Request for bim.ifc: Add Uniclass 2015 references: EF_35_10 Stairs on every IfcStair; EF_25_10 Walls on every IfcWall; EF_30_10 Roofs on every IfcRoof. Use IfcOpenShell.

First a look at what the model holds.

```python
import ifcopenshell

model = ifcopenshell.open("bim.ifc")
print(model.schema)
print("classifications:", [c.Name for c in model.by_type("IfcClassification")])
for ifc_class in ("IfcDoor", "IfcRoof", "IfcStair", "IfcWall", "IfcWindow"):
    print(ifc_class, len(model.by_type(ifc_class)))
```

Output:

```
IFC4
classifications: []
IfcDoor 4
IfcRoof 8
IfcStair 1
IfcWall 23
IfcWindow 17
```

```python
import ifcopenshell
import ifcopenshell.api.classification

model = ifcopenshell.open("bim.ifc")

system = ifcopenshell.api.classification.add_classification(model, classification="Uniclass 2015")

codes = {
    "IfcStair": ("EF_35_10", "Stairs"),
    "IfcWall": ("EF_25_10", "Walls"),
    "IfcRoof": ("EF_30_10", "Roofs"),
}
for ifc_class, (code, name) in codes.items():
    products = model.by_type(ifc_class)
    ifcopenshell.api.classification.add_reference(
        model, products=products, classification=system, identification=code, name=name
    )
    print(code, len(products))

model.write("bim-out.ifc")
```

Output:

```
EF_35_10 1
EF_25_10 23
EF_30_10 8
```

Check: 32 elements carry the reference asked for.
